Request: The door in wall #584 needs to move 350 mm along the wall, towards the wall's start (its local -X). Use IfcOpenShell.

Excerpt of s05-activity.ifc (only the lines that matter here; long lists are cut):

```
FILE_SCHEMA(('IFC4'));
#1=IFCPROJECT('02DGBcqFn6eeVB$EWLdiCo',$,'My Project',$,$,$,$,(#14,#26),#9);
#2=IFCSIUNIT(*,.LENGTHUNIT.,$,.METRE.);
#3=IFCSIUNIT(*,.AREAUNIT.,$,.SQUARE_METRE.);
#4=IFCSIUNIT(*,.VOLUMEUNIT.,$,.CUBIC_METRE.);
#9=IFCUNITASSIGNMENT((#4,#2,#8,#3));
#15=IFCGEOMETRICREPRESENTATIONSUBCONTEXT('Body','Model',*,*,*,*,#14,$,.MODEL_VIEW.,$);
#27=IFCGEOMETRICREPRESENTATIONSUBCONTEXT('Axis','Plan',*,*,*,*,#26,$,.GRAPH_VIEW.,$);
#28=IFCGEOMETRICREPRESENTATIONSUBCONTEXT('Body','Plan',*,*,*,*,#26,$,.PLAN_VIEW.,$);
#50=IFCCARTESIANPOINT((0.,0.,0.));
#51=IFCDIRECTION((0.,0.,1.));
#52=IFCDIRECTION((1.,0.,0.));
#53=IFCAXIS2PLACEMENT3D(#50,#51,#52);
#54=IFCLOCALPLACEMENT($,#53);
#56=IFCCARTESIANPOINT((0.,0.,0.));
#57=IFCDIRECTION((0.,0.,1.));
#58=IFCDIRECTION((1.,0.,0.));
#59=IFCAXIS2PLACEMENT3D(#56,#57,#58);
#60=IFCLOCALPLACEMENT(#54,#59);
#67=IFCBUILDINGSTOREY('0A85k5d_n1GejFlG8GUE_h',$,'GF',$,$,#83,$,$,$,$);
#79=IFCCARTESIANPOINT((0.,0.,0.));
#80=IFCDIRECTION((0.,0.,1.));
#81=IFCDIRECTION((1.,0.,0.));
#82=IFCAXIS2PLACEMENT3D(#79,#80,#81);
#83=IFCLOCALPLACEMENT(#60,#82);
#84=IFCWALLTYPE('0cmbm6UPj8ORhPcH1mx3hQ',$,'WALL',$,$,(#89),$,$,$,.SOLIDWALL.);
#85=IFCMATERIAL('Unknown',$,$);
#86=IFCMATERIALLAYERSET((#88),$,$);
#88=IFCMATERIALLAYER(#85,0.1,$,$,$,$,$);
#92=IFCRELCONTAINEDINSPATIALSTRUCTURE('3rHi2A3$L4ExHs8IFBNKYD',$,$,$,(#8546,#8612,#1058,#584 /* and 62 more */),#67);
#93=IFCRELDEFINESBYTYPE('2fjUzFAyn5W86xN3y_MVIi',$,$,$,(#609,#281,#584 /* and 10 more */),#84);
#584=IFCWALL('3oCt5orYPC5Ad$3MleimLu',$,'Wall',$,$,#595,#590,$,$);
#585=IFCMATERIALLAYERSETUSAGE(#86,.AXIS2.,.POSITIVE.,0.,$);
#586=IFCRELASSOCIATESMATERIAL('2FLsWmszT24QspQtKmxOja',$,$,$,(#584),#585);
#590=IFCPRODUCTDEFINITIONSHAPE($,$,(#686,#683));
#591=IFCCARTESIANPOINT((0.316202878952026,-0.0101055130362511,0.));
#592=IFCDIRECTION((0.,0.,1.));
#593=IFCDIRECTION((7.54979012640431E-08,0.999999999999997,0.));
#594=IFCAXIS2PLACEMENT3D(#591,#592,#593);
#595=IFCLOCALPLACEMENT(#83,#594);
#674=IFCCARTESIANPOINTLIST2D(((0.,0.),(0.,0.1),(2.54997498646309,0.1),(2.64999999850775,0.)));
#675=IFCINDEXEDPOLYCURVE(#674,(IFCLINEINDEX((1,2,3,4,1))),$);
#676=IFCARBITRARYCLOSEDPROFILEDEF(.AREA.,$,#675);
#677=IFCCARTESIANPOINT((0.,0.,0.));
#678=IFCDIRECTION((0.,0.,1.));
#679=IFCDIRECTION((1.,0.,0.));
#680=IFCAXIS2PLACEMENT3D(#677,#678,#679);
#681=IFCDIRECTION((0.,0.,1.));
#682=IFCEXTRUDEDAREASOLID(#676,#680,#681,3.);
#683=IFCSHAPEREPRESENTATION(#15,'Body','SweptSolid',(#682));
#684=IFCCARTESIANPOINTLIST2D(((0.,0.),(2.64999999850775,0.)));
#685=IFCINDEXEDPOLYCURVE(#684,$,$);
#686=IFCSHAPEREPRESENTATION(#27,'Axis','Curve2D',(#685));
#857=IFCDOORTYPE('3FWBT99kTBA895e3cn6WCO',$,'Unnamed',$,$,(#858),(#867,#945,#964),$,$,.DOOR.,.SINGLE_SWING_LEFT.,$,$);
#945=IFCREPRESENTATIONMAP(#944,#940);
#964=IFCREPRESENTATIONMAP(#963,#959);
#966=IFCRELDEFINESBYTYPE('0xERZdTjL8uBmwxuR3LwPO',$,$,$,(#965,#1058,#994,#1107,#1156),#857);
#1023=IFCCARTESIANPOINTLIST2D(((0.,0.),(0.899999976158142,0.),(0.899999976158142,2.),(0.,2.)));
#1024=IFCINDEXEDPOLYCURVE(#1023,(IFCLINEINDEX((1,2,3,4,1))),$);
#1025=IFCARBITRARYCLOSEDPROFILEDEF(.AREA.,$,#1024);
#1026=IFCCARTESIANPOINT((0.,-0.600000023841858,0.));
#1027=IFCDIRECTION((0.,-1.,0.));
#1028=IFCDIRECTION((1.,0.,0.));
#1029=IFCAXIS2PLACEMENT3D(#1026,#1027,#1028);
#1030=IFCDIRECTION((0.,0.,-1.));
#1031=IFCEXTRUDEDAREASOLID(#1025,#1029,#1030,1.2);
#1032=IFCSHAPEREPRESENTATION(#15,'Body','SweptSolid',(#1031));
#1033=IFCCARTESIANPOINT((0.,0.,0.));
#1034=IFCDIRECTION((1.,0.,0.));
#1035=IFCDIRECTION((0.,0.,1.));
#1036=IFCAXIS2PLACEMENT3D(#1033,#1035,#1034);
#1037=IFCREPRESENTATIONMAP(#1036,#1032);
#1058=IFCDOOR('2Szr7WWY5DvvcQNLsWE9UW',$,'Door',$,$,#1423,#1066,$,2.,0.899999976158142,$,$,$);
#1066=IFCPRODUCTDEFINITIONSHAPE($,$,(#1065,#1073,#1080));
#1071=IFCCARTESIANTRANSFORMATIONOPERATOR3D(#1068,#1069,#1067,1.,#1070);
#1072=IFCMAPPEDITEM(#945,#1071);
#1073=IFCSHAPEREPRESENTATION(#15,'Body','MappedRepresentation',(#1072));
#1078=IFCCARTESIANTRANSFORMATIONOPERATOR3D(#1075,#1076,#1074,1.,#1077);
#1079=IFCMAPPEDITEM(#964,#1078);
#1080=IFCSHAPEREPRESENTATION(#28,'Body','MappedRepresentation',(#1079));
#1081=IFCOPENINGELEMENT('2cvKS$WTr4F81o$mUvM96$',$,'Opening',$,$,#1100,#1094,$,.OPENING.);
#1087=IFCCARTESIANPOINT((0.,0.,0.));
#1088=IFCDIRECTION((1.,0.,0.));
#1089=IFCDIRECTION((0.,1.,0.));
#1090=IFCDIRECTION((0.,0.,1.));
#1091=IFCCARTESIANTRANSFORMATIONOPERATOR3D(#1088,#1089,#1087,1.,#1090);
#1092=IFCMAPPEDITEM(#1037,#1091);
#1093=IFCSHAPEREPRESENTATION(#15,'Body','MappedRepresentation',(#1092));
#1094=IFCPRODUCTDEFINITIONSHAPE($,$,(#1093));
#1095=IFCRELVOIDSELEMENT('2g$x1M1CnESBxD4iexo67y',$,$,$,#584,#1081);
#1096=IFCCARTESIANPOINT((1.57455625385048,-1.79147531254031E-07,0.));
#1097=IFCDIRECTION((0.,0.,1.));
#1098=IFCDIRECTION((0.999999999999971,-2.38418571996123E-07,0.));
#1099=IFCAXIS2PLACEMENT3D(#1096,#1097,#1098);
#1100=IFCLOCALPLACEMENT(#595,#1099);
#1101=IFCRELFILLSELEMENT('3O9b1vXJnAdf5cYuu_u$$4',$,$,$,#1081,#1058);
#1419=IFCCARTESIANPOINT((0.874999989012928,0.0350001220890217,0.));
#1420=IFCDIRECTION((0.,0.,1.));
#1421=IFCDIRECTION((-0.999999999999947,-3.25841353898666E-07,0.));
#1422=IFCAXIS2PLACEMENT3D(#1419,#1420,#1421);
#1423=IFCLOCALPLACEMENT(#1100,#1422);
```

```python
import ifcopenshell
import ifcopenshell.api.geometry
import ifcopenshell.util.placement
import ifcopenshell.util.unit

model = ifcopenshell.open("s05-activity.ifc")
unit_scale = ifcopenshell.util.unit.calculate_unit_scale(model)

door = model.by_guid("2Szr7WWY5DvvcQNLsWE9UW")
opening = door.FillsVoids[0].RelatingOpeningElement
wall = opening.VoidsElements[0].RelatingBuildingElement

wall_matrix = ifcopenshell.util.placement.get_local_placement(wall.ObjectPlacement)
shift = wall_matrix[:3, 0] * -0.35 / unit_scale
before = ifcopenshell.util.placement.get_local_placement(door.ObjectPlacement)[:3, 3].copy()

# The door is placed relative to its opening, so it follows when the opening moves.
matrix = ifcopenshell.util.placement.get_local_placement(opening.ObjectPlacement)
matrix[:3, 3] += shift
ifcopenshell.api.geometry.edit_object_placement(
    model, product=opening, matrix=matrix, is_si=False, should_transform_children=True
)

after = ifcopenshell.util.placement.get_local_placement(door.ObjectPlacement)[:3, 3]
print("door moved by", (after - before).round(3) + 0.0)

model.write("s05-activity_edited.ifc")
```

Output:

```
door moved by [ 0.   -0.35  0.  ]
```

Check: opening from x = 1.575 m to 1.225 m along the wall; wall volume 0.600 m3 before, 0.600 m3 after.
